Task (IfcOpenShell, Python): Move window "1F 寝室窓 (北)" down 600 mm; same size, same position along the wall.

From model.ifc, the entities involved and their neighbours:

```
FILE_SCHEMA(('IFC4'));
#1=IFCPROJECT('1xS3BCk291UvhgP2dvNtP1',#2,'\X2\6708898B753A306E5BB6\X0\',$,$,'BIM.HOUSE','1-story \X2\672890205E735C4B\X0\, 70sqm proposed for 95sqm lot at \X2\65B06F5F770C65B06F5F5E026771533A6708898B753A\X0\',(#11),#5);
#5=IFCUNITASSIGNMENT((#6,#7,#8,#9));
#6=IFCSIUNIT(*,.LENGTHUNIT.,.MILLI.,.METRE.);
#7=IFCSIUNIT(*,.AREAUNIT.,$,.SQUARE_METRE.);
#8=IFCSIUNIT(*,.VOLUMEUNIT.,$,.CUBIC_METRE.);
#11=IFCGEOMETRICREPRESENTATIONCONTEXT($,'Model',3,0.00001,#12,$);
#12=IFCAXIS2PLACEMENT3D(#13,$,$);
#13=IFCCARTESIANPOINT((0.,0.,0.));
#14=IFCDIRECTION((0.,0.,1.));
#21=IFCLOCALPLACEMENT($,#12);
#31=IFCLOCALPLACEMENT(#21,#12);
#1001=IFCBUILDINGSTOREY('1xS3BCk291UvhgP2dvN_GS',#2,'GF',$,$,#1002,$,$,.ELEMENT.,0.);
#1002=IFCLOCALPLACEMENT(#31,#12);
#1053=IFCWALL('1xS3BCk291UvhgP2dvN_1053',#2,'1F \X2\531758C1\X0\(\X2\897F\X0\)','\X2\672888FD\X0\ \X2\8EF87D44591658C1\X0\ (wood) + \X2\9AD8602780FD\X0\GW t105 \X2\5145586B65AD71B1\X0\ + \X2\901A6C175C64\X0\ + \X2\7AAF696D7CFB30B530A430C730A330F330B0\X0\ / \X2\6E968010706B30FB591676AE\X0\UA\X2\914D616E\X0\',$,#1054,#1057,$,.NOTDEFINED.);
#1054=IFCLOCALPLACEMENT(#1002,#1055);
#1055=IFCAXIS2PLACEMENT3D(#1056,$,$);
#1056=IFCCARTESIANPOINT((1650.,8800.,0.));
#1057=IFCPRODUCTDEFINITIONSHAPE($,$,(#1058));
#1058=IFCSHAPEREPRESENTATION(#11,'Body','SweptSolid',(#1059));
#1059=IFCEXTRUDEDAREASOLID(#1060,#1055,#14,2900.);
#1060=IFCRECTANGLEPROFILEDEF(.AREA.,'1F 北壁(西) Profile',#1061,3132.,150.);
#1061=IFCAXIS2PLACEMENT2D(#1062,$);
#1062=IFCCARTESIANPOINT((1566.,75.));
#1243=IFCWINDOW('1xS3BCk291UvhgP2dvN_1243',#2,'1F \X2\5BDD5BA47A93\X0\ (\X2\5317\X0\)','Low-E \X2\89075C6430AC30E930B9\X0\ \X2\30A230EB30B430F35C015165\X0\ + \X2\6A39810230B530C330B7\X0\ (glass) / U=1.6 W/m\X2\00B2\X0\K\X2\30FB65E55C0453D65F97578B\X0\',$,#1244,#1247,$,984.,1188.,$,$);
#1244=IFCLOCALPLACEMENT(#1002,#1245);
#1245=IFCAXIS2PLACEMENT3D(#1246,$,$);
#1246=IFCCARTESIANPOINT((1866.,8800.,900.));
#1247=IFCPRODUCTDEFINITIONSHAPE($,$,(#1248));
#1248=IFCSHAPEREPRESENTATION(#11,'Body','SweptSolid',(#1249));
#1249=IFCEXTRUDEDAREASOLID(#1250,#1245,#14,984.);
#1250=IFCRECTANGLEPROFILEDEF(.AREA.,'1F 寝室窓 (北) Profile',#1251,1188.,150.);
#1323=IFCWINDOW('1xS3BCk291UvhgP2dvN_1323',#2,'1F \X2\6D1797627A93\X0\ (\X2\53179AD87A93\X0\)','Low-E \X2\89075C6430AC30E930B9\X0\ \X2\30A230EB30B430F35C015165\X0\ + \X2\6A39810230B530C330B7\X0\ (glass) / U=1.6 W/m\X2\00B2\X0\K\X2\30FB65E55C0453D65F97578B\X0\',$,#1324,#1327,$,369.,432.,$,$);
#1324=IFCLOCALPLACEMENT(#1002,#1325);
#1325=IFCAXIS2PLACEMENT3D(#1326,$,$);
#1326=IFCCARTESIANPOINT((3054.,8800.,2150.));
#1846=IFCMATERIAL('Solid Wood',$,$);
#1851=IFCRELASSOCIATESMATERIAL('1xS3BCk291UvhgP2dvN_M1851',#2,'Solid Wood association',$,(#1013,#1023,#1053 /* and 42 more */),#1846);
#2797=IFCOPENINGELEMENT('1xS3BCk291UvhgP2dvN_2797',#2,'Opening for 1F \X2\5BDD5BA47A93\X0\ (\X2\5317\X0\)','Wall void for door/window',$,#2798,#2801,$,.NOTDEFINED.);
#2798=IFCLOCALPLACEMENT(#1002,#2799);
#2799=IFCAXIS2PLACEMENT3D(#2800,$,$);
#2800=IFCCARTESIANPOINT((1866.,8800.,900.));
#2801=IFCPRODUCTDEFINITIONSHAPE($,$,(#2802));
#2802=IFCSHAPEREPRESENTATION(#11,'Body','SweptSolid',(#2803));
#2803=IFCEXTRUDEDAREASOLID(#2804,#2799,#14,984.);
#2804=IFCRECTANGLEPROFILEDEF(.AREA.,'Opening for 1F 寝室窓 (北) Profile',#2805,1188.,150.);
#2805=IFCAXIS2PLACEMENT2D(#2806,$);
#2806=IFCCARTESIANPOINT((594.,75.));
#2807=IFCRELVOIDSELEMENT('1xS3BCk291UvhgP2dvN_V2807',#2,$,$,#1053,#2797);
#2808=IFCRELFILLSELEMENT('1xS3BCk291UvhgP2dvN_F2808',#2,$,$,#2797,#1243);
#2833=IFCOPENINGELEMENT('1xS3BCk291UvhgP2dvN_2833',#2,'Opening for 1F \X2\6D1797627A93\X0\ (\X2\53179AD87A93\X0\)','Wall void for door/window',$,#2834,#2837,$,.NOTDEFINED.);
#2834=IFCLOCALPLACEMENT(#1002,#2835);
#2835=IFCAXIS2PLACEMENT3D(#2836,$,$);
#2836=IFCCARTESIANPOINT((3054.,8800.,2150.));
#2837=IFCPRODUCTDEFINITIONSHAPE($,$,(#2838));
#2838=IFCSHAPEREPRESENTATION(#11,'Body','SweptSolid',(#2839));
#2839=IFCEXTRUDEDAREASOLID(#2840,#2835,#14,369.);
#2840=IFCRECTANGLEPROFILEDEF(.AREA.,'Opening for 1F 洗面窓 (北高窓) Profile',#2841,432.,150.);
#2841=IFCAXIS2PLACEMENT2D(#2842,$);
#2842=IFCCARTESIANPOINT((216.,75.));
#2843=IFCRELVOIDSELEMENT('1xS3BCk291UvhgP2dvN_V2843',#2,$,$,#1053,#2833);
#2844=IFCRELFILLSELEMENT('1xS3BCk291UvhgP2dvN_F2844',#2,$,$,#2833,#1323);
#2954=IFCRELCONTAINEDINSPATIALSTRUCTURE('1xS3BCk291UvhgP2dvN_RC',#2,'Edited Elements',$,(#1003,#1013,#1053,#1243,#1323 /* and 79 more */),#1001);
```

```python
import numpy as np
import ifcopenshell
import ifcopenshell.api.geometry
import ifcopenshell.util.placement
import ifcopenshell.util.unit

model = ifcopenshell.open("model.ifc")
unit_scale = ifcopenshell.util.unit.calculate_unit_scale(model)

window = model.by_guid("1xS3BCk291UvhgP2dvN_1243")
opening = window.FillsVoids[0].RelatingOpeningElement
dz = -600.0

shift = np.array([0.0, 0.0, dz])
# The window is not placed relative to its opening, so move both.
for product in (opening, window):
    matrix = ifcopenshell.util.placement.get_local_placement(product.ObjectPlacement)
    matrix[:3, 3] += shift
    ifcopenshell.api.geometry.edit_object_placement(model, product=product, matrix=matrix, is_si=False)

print(f"moved by {dz * unit_scale:+.3f} m")

model.write("model_edited.ifc")
```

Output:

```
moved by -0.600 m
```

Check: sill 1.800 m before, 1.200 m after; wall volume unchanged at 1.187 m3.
